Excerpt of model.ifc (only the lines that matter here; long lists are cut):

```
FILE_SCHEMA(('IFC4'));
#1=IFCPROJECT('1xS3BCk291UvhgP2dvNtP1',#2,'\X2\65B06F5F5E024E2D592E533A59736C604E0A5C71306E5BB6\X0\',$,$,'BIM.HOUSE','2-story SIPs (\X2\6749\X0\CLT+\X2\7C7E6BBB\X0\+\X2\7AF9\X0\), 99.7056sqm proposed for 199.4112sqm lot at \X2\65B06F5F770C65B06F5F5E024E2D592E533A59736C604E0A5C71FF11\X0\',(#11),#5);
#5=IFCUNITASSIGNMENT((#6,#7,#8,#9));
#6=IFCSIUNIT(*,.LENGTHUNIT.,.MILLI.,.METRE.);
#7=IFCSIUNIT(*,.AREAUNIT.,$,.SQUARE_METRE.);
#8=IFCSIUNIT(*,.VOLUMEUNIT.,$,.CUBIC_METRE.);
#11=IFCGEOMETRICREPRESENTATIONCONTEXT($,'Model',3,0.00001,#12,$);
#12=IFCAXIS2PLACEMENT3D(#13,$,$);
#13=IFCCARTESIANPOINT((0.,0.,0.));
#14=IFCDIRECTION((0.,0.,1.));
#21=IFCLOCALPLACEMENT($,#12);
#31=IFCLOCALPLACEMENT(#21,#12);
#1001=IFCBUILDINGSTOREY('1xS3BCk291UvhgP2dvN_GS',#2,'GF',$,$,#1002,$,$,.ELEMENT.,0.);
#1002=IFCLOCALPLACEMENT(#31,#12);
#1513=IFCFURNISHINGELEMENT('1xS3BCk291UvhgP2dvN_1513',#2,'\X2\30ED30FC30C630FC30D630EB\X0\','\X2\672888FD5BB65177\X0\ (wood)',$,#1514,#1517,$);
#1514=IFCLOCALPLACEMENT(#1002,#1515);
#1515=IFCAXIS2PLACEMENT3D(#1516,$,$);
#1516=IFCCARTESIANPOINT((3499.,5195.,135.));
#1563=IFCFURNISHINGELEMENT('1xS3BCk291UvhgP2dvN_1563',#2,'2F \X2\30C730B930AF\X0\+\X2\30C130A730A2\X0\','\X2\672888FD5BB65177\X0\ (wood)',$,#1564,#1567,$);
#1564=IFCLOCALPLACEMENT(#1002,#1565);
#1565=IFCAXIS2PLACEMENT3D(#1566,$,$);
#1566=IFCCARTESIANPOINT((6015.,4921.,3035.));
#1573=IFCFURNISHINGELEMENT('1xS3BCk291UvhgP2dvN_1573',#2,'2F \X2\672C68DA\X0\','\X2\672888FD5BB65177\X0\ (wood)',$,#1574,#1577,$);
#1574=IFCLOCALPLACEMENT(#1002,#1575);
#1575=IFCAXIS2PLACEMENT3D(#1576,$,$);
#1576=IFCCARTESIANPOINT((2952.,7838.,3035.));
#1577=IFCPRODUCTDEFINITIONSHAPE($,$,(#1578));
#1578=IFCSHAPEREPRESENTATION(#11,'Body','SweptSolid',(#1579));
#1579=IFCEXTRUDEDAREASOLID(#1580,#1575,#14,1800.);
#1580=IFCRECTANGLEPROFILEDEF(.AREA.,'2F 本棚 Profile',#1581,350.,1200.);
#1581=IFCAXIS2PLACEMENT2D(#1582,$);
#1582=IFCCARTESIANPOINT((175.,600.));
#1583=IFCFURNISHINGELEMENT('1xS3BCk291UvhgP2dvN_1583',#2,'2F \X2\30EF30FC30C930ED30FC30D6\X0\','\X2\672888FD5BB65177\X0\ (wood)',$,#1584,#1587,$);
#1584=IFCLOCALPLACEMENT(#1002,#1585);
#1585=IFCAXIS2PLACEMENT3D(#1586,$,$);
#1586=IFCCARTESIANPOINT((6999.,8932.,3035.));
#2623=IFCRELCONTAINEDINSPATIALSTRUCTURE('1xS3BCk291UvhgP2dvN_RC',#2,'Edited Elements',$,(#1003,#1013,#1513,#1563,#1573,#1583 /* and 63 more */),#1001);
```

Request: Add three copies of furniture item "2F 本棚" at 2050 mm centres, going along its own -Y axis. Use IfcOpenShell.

```python
import ifcopenshell
import ifcopenshell.api.geometry
import ifcopenshell.api.root
import ifcopenshell.util.element
import ifcopenshell.util.placement
import ifcopenshell.util.unit

model = ifcopenshell.open("model.ifc")
unit_scale = ifcopenshell.util.unit.calculate_unit_scale(model)


def reuse_history(source, copy):
    """copy_class also copies each property set's owner history, people and application; keep the originals."""
    for rel in copy.IsDefinedBy:
        if rel.is_a("IfcRelDefinesByProperties") and (history := rel.RelatingPropertyDefinition.OwnerHistory):
            rel.RelatingPropertyDefinition.OwnerHistory = source.OwnerHistory
            ifcopenshell.util.element.remove_deep2(model, history)


source = model.by_guid("1xS3BCk291UvhgP2dvN_1573")
base = ifcopenshell.util.placement.get_local_placement(source.ObjectPlacement)
step = -base[:3, 1] * 2.05 / unit_scale

for i in range(1, 4):
    copy = ifcopenshell.api.root.copy_class(model, product=source)
    copy.Representation = ifcopenshell.util.element.copy_deep(
        model, source.Representation, exclude=["IfcGeometricRepresentationContext", "IfcRepresentationMap"]
    )
    reuse_history(source, copy)
    matrix = base.copy()
    matrix[:3, 3] += i * step
    print("added at", matrix[:3, 3].round(3) + 0.0)
    ifcopenshell.api.geometry.edit_object_placement(model, product=copy, matrix=matrix, is_si=False)

model.write("model_edited.ifc")
```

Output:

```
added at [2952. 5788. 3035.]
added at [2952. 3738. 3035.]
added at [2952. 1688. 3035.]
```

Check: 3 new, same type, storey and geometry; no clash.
